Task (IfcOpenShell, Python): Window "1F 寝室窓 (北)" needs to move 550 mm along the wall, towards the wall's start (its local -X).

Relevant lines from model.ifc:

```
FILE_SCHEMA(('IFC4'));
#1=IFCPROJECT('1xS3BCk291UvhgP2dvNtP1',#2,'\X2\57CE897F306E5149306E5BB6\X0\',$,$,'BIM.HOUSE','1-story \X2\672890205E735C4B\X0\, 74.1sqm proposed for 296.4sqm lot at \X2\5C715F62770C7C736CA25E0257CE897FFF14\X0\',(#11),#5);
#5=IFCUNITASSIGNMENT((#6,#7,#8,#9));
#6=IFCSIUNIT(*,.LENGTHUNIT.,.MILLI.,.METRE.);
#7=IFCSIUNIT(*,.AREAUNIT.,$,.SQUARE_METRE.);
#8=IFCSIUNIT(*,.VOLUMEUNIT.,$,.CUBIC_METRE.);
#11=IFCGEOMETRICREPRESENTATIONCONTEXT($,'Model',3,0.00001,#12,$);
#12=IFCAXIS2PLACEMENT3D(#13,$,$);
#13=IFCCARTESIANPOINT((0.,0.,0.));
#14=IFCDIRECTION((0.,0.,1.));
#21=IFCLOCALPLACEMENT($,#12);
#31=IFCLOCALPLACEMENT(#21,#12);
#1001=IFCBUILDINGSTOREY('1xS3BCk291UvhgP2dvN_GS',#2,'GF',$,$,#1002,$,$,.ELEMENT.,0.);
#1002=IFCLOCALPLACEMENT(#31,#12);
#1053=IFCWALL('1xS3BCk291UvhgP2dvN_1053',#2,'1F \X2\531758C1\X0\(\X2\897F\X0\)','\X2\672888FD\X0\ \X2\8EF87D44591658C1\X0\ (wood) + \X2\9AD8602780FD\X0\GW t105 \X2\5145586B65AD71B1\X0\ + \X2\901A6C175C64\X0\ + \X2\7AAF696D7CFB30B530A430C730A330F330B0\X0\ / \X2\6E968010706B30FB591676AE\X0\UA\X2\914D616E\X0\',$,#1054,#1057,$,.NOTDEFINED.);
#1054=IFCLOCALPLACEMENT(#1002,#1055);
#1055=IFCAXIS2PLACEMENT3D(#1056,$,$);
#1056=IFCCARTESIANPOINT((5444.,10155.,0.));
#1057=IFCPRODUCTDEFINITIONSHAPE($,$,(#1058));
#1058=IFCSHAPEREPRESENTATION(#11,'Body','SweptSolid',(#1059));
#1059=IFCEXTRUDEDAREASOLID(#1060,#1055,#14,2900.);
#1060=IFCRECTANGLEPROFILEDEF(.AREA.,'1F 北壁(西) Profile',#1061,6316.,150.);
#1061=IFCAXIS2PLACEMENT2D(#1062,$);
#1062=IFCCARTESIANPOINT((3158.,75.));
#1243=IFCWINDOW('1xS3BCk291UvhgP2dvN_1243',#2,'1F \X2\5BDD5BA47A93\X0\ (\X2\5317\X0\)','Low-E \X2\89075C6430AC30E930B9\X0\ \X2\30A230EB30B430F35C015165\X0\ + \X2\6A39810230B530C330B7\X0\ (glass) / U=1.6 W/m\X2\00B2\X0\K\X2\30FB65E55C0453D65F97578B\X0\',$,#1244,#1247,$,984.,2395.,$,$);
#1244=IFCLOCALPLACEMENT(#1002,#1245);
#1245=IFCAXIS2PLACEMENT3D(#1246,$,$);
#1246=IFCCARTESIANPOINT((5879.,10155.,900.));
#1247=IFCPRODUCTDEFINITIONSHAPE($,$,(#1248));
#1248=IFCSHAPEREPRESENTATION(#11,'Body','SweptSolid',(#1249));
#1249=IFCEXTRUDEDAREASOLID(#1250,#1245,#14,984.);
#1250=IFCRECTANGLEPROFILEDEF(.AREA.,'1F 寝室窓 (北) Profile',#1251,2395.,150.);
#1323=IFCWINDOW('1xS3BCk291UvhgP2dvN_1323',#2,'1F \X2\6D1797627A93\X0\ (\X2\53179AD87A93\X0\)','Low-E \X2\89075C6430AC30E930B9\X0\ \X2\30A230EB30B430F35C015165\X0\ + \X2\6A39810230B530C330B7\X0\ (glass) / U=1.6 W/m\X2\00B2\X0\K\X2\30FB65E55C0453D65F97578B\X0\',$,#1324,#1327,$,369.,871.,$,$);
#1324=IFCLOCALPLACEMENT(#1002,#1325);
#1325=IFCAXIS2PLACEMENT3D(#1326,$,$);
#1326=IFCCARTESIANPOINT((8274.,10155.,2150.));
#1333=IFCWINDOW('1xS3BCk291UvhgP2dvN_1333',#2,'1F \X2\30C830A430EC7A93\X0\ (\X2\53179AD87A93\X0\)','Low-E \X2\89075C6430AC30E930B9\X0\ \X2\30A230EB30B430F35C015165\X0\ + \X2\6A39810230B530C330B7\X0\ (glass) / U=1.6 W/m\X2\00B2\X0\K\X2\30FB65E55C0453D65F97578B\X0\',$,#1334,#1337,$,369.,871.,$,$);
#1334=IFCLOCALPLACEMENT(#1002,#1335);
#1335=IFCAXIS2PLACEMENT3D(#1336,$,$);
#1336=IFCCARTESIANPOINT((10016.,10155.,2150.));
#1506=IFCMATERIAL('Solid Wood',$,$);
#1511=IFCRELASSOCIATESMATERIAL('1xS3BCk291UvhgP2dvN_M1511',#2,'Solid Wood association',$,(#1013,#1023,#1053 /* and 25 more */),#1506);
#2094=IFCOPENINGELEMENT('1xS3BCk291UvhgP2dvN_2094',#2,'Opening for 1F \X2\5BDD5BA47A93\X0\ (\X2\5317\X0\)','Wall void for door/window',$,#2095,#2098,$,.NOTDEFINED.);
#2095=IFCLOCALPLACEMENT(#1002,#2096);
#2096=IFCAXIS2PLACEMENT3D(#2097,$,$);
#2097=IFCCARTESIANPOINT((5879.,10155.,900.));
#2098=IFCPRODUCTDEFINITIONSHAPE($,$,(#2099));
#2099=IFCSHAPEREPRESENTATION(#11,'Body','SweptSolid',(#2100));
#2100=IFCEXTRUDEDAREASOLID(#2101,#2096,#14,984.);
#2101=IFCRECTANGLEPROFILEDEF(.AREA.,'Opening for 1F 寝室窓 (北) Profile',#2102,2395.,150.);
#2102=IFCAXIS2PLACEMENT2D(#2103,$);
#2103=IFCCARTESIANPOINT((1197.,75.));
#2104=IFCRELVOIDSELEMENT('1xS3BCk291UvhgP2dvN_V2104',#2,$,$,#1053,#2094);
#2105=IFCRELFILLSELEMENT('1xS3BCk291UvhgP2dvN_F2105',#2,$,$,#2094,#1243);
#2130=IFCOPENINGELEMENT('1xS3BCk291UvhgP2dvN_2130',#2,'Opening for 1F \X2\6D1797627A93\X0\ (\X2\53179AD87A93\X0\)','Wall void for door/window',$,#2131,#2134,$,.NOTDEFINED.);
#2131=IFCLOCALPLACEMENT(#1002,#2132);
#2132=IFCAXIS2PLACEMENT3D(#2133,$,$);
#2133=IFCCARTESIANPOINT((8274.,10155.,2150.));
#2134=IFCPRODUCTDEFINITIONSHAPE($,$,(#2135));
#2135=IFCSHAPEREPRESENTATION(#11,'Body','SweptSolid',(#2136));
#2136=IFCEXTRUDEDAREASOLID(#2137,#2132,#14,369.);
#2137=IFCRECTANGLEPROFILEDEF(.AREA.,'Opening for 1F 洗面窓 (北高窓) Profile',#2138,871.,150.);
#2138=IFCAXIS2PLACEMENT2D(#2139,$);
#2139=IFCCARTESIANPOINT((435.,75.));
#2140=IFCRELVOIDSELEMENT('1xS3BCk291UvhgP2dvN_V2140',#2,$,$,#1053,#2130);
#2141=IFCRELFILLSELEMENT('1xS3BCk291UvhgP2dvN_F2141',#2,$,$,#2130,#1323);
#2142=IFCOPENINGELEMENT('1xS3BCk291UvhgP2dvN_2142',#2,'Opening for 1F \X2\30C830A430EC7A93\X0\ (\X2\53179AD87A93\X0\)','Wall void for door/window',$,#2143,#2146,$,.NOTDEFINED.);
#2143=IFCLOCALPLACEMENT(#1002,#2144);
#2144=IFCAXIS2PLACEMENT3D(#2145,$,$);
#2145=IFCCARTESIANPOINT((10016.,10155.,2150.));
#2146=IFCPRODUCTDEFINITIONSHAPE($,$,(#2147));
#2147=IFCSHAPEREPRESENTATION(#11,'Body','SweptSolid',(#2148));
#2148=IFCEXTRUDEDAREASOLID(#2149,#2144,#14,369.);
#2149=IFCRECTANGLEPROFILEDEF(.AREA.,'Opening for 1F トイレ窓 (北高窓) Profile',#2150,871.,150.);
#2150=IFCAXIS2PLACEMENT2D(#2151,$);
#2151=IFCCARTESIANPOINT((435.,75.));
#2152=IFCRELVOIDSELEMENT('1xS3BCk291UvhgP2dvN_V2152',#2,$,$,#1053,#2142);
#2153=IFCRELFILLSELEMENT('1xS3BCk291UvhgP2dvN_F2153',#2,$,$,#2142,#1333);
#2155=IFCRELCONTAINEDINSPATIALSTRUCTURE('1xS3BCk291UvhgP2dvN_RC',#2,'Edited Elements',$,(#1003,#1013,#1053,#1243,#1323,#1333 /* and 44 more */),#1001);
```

```python
import ifcopenshell
import ifcopenshell.api.geometry
import ifcopenshell.util.placement
import ifcopenshell.util.unit

model = ifcopenshell.open("model.ifc")
unit_scale = ifcopenshell.util.unit.calculate_unit_scale(model)

window = model.by_id(1243)
opening = window.FillsVoids[0].RelatingOpeningElement
wall = opening.VoidsElements[0].RelatingBuildingElement

wall_matrix = ifcopenshell.util.placement.get_local_placement(wall.ObjectPlacement)
shift = wall_matrix[:3, 0] * -0.55 / unit_scale
before = ifcopenshell.util.placement.get_local_placement(window.ObjectPlacement)[:3, 3].copy()

# The window is not placed relative to its opening, so move both.
for product in (opening, window):
    matrix = ifcopenshell.util.placement.get_local_placement(product.ObjectPlacement)
    matrix[:3, 3] += shift
    ifcopenshell.api.geometry.edit_object_placement(model, product=product, matrix=matrix, is_si=False)

after = ifcopenshell.util.placement.get_local_placement(window.ObjectPlacement)[:3, 3]
print("window moved by", (after - before).round(3) + 0.0)

model.write("model_rev.ifc")
```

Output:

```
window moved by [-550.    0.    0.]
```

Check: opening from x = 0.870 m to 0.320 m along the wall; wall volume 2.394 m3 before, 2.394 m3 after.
